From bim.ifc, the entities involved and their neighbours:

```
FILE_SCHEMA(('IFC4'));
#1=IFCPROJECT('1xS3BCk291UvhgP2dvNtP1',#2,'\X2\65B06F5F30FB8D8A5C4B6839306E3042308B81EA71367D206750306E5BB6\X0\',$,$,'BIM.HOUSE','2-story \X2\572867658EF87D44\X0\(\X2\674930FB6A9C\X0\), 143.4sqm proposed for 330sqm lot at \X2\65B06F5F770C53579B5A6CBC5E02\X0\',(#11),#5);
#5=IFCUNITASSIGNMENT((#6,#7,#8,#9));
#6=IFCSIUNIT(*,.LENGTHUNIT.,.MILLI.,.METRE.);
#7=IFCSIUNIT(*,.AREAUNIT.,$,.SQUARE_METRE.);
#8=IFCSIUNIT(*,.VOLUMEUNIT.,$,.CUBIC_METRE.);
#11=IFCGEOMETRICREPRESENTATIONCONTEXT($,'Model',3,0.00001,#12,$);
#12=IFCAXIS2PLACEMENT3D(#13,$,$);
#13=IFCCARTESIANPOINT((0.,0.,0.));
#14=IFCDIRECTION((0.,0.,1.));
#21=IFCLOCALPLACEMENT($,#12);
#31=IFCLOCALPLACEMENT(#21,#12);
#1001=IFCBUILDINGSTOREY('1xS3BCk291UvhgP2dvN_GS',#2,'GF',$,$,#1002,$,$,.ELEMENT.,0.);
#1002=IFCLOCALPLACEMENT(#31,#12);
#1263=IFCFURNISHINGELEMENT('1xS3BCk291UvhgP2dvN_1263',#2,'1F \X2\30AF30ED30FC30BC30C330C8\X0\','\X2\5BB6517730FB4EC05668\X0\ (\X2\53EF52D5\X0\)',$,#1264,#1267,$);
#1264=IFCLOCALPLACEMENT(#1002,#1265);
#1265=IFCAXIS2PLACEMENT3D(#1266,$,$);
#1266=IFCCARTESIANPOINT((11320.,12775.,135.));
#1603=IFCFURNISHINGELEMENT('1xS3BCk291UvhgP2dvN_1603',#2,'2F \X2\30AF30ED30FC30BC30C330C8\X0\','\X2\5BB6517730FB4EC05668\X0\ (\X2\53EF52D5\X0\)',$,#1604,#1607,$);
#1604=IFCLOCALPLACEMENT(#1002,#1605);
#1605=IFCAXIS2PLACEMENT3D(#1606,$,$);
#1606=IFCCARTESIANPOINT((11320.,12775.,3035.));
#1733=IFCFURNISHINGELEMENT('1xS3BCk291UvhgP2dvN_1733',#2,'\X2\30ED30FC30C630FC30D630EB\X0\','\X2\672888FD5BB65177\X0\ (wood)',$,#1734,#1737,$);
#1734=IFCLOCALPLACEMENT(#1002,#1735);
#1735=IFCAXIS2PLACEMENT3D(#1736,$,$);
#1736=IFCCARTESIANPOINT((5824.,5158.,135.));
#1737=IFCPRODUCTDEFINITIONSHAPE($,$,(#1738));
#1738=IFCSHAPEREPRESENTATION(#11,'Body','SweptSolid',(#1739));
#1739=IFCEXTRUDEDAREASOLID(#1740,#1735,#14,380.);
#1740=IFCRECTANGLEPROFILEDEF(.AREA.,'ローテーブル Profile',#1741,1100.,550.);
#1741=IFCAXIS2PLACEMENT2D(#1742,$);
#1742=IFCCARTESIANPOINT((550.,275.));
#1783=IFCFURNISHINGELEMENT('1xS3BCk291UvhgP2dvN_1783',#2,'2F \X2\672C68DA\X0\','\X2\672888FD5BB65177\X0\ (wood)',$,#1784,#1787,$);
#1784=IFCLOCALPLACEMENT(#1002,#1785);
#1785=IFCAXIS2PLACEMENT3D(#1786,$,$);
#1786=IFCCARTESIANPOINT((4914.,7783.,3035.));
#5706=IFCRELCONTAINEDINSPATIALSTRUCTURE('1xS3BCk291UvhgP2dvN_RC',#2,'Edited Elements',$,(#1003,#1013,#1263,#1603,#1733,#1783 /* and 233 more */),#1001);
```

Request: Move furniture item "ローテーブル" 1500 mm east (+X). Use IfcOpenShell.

```python
import ifcopenshell
import ifcopenshell.api.geometry
import ifcopenshell.util.placement
import ifcopenshell.util.unit

model = ifcopenshell.open("bim.ifc")
unit_scale = ifcopenshell.util.unit.calculate_unit_scale(model)

item = model.by_id(1733)
matrix = ifcopenshell.util.placement.get_local_placement(item.ObjectPlacement)
matrix[0, 3] += 1.5 / unit_scale
ifcopenshell.api.geometry.edit_object_placement(model, product=item, matrix=matrix, is_si=False)

print(ifcopenshell.util.placement.get_local_placement(item.ObjectPlacement).round(3) + 0.0)

model.write("bim_updated.ifc")
```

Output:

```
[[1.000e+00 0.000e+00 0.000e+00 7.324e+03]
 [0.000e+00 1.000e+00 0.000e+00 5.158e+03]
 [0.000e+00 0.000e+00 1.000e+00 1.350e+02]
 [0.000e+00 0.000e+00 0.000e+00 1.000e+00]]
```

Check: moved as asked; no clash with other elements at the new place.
